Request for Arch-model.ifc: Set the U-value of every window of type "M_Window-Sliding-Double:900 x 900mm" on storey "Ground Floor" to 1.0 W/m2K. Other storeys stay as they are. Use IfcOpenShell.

First a look at what the model holds.

```python
import ifcopenshell
import ifcopenshell.util.element

model = ifcopenshell.open("Arch-model.ifc")
print(model.schema)
storey = next(s for s in model.by_type("IfcBuildingStorey") if s.Name == "Ground Floor")
windows = [e for e in ifcopenshell.util.element.get_decomposition(storey) if e.is_a("IfcWindow")]
seen = {}
for e in windows:
    element_type = ifcopenshell.util.element.get_type(e)
    key = (element_type.Name if element_type != e and element_type else None, ifcopenshell.util.element.get_pset(e, "Pset_WindowCommon", "ThermalTransmittance"))
    seen[key] = seen.get(key, 0) + 1
for (name, value), count in sorted(seen.items(), key=str):
    print(count, "x", name, "|", value)
```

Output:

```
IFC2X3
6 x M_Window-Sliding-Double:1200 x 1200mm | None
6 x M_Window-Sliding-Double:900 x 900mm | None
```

```python
import ifcopenshell
import ifcopenshell.api.pset
import ifcopenshell.util.element

model = ifcopenshell.open("Arch-model.ifc")

storey = next(s for s in model.by_type("IfcBuildingStorey") if s.Name == "Ground Floor")
windows = [e for e in ifcopenshell.util.element.get_decomposition(storey) if e.is_a("IfcWindow")]

count = 0
for e in windows:
    element_type = ifcopenshell.util.element.get_type(e)
    if element_type in (None, e) or element_type.Name != "M_Window-Sliding-Double:900 x 900mm":
        continue
    # add_pset returns the element's existing set when there is one.
    pset = ifcopenshell.api.pset.add_pset(model, product=e, name="Pset_WindowCommon")
    ifcopenshell.api.pset.edit_pset(model, pset=pset, properties={"ThermalTransmittance": 1.0})
    count += 1

print(count, "windows updated")

model.write("Arch-model_edited.ifc")
```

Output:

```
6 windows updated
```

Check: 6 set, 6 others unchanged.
